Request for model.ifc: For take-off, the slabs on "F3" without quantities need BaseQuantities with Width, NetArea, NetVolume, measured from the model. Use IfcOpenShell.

First a look at what the model holds.

```python
import ifcopenshell
import ifcopenshell.util.element
import ifcopenshell.util.unit

model = ifcopenshell.open("model.ifc")
print(model.schema)
for unit_type in ("LENGTHUNIT", "AREAUNIT", "VOLUMEUNIT"):
    print(unit_type, ifcopenshell.util.unit.calculate_unit_scale(model, unit_type))
storey = next(s for s in model.by_type("IfcBuildingStorey") if s.Name == "F3")
slabs = [e for e in ifcopenshell.util.element.get_decomposition(storey) if e.is_a("IfcSlab")]
for e in sorted(slabs, key=lambda e: e.id()):
    print(e.id(), e.is_a(), e.Name, list(ifcopenshell.util.element.get_psets(e, qtos_only=True)), sep=" | ")
```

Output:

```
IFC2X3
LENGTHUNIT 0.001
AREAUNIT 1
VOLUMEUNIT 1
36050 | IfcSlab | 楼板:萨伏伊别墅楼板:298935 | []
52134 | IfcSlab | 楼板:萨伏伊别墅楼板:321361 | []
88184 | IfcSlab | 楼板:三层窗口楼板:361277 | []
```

```python
import ifcopenshell
import ifcopenshell.api.pset
import ifcopenshell.geom
import ifcopenshell.util.element
import ifcopenshell.util.shape
import ifcopenshell.util.unit

model = ifcopenshell.open("model.ifc")
unit_scale = ifcopenshell.util.unit.calculate_unit_scale(model)
area_scale = ifcopenshell.util.unit.calculate_unit_scale(model, "AREAUNIT")
volume_scale = ifcopenshell.util.unit.calculate_unit_scale(model, "VOLUMEUNIT")
settings = ifcopenshell.geom.settings()

storey = next(s for s in model.by_type("IfcBuildingStorey") if s.Name == "F3")
slabs = [e for e in ifcopenshell.util.element.get_decomposition(storey) if e.is_a("IfcSlab")]

for e in sorted(slabs, key=lambda e: e.id()):
    if ifcopenshell.util.element.get_psets(e, qtos_only=True, should_inherit=False):
        continue
    # Geometry comes back in metres, in the element's own axes.
    shape = ifcopenshell.geom.create_shape(settings, e)
    values = {
        "Width": ifcopenshell.util.shape.get_z(shape.geometry) / unit_scale,
        "NetArea": ifcopenshell.util.shape.get_footprint_area(shape.geometry) / area_scale,
        "NetVolume": ifcopenshell.util.shape.get_volume(shape.geometry) / volume_scale,
    }
    qto = ifcopenshell.api.pset.add_qto(model, product=e, name="BaseQuantities")
    ifcopenshell.api.pset.edit_qto(model, qto=qto, properties=values)
    print(e.id(), {k: round(v, 3) for k, v in values.items()})

model.write("model_edited.ifc")
```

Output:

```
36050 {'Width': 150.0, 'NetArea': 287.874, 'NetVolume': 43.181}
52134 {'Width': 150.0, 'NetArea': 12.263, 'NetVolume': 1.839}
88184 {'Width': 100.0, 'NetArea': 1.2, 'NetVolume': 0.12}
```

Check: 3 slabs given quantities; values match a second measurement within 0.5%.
